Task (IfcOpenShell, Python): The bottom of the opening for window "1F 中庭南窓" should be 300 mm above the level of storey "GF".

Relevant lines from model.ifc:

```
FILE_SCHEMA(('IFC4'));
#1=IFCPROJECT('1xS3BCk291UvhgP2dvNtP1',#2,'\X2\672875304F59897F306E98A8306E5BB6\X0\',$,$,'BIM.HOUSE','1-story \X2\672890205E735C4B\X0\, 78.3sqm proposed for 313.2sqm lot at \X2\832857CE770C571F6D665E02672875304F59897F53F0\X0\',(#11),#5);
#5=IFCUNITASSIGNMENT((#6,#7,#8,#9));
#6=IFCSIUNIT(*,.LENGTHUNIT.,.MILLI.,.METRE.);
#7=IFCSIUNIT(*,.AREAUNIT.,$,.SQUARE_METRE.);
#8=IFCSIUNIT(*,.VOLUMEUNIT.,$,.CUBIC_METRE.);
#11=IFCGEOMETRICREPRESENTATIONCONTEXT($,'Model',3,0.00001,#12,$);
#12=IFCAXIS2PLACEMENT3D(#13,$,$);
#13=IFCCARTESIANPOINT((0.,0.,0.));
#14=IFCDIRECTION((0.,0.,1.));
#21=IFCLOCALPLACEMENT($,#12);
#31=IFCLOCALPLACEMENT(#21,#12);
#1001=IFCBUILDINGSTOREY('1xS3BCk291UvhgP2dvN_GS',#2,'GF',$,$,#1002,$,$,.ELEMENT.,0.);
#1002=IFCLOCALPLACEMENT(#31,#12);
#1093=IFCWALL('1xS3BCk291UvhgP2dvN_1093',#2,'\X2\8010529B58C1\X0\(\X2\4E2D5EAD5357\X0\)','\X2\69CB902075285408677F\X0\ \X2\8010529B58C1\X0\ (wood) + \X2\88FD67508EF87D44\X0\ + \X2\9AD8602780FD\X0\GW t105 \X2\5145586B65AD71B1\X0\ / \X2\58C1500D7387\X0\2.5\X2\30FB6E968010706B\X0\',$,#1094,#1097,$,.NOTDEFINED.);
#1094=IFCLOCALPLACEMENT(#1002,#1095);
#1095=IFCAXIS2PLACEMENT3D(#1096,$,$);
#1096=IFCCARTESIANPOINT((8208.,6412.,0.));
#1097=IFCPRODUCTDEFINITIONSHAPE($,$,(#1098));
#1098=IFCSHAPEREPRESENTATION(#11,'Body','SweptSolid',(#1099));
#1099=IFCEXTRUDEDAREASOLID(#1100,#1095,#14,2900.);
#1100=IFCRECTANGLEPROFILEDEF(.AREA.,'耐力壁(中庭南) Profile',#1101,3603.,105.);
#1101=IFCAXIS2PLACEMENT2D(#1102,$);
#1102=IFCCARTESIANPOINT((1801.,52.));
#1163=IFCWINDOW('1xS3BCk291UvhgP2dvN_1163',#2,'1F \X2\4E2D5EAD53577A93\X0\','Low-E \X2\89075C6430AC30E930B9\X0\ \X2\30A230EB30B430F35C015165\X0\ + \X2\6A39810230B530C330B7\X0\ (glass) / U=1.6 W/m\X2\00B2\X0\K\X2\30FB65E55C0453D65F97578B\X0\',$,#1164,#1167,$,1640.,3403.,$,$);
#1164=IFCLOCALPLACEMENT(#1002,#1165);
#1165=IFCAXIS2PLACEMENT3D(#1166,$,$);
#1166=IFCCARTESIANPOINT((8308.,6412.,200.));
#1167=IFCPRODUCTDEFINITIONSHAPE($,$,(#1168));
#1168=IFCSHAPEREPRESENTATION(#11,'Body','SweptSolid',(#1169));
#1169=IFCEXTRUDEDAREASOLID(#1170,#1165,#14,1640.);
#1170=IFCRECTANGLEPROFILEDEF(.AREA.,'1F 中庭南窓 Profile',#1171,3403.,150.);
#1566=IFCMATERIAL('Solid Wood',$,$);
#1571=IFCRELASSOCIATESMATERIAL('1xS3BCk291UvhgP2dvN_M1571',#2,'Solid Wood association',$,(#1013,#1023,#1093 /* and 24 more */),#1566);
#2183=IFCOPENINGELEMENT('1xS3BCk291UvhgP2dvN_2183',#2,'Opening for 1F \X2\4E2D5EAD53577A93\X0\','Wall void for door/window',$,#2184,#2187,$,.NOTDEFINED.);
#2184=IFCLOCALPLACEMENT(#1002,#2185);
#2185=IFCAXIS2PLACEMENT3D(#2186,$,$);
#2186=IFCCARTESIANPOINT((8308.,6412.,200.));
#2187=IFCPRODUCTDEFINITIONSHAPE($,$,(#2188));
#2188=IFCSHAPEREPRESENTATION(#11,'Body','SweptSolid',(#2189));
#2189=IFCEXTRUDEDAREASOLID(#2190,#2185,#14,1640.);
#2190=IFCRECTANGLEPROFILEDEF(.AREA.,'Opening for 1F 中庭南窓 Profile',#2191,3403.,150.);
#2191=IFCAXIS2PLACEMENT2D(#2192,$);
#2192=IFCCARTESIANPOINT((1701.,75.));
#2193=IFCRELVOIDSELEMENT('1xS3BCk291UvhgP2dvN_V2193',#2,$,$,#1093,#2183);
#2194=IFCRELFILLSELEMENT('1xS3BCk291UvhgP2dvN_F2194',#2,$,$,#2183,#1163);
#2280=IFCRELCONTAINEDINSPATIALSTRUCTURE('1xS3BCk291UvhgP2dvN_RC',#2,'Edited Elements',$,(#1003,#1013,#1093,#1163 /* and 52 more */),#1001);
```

```python
import numpy as np
import ifcopenshell
import ifcopenshell.api.geometry
import ifcopenshell.geom
import ifcopenshell.util.element
import ifcopenshell.util.placement
import ifcopenshell.util.shape
import ifcopenshell.util.unit

model = ifcopenshell.open("model.ifc")
unit_scale = ifcopenshell.util.unit.calculate_unit_scale(model)

window = model.by_guid("1xS3BCk291UvhgP2dvN_1163")
opening = window.FillsVoids[0].RelatingOpeningElement
storey = ifcopenshell.util.element.get_container(window, ifc_class="IfcBuildingStorey")
level = ifcopenshell.util.placement.get_local_placement(storey.ObjectPlacement)[2, 3]

# The opening's origin need not be at the sill, so measure its lowest point.
shape = ifcopenshell.geom.create_shape(ifcopenshell.geom.settings(), opening)
bottom = ifcopenshell.util.shape.get_shape_bottom_elevation(shape, shape.geometry) / unit_scale
dz = level + 0.3 / unit_scale - bottom

shift = np.array([0.0, 0.0, dz])
# The window is not placed relative to its opening, so move both.
for product in (opening, window):
    matrix = ifcopenshell.util.placement.get_local_placement(product.ObjectPlacement)
    matrix[:3, 3] += shift
    ifcopenshell.api.geometry.edit_object_placement(model, product=product, matrix=matrix, is_si=False)

print(f"moved by {dz * unit_scale:+.3f} m")

model.write("model-out.ifc")
```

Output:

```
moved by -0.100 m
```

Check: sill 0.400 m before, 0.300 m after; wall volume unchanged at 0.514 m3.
